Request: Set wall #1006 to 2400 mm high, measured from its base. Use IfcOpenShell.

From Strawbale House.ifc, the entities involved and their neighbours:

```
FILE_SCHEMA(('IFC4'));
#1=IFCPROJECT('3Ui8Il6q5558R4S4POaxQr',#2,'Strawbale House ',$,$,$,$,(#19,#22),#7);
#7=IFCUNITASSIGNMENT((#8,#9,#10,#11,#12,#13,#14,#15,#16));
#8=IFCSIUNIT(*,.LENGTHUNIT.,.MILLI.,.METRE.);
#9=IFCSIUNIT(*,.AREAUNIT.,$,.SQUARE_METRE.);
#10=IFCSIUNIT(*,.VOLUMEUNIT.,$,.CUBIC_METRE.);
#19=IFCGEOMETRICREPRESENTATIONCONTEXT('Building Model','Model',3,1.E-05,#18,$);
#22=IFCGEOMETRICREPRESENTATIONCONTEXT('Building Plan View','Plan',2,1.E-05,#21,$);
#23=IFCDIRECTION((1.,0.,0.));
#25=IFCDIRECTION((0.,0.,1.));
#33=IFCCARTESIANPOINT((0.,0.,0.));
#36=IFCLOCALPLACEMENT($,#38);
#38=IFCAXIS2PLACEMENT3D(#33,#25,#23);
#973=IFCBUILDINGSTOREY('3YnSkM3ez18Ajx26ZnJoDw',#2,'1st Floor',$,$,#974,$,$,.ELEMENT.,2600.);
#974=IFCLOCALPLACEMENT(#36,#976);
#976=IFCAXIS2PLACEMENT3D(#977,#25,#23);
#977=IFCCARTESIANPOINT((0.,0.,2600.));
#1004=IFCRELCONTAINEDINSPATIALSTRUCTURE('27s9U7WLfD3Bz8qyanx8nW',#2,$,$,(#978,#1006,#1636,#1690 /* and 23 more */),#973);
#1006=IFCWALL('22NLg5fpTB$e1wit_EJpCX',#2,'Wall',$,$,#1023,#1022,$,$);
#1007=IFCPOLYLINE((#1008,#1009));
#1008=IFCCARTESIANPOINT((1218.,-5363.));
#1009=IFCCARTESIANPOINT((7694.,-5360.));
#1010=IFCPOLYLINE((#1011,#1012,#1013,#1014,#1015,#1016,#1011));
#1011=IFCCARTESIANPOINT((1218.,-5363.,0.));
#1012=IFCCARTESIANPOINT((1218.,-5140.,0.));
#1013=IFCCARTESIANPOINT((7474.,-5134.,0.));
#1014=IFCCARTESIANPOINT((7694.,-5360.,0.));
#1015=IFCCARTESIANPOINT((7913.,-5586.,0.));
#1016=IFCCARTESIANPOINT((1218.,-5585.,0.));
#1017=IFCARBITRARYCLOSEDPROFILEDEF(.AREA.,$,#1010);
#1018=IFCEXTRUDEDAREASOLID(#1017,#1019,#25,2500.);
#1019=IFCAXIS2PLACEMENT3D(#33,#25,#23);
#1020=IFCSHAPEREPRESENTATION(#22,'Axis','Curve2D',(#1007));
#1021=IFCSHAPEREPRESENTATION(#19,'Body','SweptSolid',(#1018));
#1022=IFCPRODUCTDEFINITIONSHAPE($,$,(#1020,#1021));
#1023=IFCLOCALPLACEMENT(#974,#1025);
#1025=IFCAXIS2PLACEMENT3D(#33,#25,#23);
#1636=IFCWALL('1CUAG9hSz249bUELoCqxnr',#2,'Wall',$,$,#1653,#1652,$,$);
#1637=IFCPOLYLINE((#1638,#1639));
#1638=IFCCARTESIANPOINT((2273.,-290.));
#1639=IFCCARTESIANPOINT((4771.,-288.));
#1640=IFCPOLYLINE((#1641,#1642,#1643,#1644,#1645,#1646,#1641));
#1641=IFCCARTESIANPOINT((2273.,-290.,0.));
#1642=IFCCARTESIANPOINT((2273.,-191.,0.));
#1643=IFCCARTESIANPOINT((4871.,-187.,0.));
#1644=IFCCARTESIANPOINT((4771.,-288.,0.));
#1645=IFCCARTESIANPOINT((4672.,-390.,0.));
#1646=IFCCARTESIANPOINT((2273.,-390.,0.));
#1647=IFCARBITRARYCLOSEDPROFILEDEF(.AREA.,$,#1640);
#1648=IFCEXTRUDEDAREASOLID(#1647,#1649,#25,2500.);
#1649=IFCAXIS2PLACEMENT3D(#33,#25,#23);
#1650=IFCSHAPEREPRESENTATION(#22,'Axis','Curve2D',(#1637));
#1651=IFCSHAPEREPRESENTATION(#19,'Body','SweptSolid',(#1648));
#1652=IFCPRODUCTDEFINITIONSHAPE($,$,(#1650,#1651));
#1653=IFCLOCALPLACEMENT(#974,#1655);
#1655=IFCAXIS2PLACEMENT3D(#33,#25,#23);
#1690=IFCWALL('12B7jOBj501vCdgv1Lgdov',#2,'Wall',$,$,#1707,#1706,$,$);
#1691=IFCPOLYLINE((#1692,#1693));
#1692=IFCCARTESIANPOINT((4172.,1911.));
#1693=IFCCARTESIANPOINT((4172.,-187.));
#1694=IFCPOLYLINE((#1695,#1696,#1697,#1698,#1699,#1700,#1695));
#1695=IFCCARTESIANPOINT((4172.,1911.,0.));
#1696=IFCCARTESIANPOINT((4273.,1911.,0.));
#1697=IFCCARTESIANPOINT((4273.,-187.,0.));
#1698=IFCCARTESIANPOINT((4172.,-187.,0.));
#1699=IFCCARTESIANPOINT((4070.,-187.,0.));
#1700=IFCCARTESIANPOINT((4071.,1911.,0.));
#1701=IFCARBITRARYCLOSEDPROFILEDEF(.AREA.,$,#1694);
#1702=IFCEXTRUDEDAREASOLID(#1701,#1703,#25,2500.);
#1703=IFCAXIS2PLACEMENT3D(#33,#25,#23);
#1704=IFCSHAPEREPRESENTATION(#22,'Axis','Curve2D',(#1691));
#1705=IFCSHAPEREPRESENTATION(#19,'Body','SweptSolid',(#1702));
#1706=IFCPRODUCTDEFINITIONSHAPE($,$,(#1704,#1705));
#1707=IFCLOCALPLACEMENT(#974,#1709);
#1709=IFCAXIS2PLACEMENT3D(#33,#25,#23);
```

```python
import ifcopenshell
import ifcopenshell.geom
import ifcopenshell.util.shape
import ifcopenshell.util.unit

model = ifcopenshell.open("Strawbale House.ifc")
unit_scale = ifcopenshell.util.unit.calculate_unit_scale(model)
settings = ifcopenshell.geom.settings()


def volume(element):
    """Net volume in cubic metres, openings subtracted."""
    shape = ifcopenshell.geom.create_shape(settings, element)
    return ifcopenshell.util.shape.get_volume(shape.geometry)


wall = model.by_guid("22NLg5fpTB$e1wit_EJpCX")
before = volume(wall)

body = next(r for r in wall.Representation.Representations if r.RepresentationIdentifier == "Body")
solid = body.Items[0]
old_height = solid.Depth
solid.Depth = 2.4 / unit_scale
after = volume(wall)

print(f"height {old_height:g} -> {solid.Depth:g}, volume {before:.3f} -> {after:.3f} m3")

model.write("Strawbale House_edited.ifc")
```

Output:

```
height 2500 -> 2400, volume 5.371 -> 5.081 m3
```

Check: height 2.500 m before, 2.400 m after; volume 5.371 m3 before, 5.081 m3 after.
